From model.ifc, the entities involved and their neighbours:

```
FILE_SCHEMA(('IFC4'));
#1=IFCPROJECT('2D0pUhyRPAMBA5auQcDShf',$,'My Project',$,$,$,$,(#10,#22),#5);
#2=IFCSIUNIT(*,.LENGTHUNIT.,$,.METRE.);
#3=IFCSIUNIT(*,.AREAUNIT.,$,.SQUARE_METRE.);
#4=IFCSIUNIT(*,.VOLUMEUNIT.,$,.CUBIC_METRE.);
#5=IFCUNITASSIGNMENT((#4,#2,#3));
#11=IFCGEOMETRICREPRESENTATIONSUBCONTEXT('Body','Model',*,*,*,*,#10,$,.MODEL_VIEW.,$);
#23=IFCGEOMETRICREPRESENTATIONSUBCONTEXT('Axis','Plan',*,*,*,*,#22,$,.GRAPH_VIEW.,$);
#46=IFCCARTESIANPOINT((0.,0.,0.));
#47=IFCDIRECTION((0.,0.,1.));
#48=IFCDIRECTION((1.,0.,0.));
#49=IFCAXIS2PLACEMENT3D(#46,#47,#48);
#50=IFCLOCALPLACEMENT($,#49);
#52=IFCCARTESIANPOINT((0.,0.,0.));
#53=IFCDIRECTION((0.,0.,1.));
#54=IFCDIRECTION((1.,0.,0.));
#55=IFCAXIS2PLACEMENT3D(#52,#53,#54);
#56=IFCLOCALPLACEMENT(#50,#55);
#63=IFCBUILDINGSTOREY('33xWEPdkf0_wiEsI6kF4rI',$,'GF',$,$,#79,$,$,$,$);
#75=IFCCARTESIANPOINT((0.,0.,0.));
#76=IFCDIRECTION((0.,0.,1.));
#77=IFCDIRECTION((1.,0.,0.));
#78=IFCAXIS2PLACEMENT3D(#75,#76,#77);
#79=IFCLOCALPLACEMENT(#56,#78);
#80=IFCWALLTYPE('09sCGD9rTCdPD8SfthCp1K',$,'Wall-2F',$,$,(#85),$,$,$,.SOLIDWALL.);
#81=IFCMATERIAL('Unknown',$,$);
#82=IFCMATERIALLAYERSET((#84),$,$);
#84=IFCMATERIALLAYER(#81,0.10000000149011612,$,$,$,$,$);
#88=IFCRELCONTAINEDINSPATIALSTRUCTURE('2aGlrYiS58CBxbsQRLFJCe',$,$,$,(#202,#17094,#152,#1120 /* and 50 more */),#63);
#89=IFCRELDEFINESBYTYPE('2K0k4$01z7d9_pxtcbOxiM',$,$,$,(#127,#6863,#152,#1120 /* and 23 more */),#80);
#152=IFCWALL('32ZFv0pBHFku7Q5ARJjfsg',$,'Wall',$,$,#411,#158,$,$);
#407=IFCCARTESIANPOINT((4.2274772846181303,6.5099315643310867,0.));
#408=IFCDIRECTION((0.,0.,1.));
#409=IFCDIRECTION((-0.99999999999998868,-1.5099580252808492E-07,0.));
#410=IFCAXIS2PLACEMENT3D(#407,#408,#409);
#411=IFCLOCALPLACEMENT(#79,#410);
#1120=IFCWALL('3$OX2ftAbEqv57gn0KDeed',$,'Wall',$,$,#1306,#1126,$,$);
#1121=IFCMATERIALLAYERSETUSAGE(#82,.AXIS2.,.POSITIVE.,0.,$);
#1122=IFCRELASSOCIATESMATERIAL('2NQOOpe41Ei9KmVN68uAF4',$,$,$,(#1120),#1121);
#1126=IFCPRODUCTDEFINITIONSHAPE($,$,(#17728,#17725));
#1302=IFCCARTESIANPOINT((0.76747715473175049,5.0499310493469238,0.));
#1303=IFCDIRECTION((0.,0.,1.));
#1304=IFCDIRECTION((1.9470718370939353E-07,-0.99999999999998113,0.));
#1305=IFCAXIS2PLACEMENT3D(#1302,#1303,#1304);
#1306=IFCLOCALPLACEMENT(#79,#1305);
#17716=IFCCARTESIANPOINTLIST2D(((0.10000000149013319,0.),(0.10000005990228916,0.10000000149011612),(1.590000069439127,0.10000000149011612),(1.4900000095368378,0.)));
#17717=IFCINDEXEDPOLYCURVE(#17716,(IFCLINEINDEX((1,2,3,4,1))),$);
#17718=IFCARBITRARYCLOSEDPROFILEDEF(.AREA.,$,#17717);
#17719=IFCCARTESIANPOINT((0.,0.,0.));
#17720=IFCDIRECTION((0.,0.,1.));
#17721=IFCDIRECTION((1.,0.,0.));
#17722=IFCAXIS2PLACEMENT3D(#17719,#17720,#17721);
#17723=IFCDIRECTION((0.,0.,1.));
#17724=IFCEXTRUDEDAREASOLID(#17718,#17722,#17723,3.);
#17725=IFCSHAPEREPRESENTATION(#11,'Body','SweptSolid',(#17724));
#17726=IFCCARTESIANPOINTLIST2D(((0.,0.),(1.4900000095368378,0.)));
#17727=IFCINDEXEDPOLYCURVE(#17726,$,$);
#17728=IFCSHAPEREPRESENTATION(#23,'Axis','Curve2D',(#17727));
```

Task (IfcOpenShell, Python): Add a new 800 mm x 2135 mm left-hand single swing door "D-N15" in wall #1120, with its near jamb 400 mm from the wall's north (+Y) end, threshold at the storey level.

```python
import numpy as np
import ifcopenshell
import ifcopenshell.api.feature
import ifcopenshell.api.geometry
import ifcopenshell.api.root
import ifcopenshell.api.spatial
import ifcopenshell.geom
import ifcopenshell.util.element
import ifcopenshell.util.placement
import ifcopenshell.util.representation
import ifcopenshell.util.shape
import ifcopenshell.util.unit

model = ifcopenshell.open("model.ifc")
unit_scale = ifcopenshell.util.unit.calculate_unit_scale(model)
settings = ifcopenshell.geom.settings()


def volume(element):
    """Net volume in cubic metres, openings subtracted."""
    shape = ifcopenshell.geom.create_shape(settings, element)
    return ifcopenshell.util.shape.get_volume(shape.geometry)


wall = model.by_guid("3$OX2ftAbEqv57gn0KDeed")
storey = ifcopenshell.util.element.get_container(wall, ifc_class="IfcBuildingStorey")
context = ifcopenshell.util.representation.get_context(model, "Model", "Body", "MODEL_VIEW")
before = volume(wall)

width, height, from_end, sill = 0.8, 2.135, 0.4, 0.0  # metres

# The wall runs along its own X axis, and the end named is its -X end.
wall_shape = ifcopenshell.geom.create_shape(settings, wall)
x, y, z = ifcopenshell.util.shape.get_vertices(wall_shape.geometry).T
start = x.min() + from_end
face, thickness = float(y.min()), float(y.max() - y.min())
wall_matrix = ifcopenshell.util.placement.get_local_placement(wall.ObjectPlacement)
level = ifcopenshell.util.placement.get_local_placement(storey.ObjectPlacement)[2, 3]


def in_wall(x, y):
    """Placement at x, y metres in the wall's axes, at sill height."""
    matrix = wall_matrix.copy()
    matrix[:, 3] = wall_matrix @ np.array([x / unit_scale, y / unit_scale, 0.0, 1.0])
    matrix[2, 3] = level + sill / unit_scale
    return matrix


# Opening: a box that overshoots both wall faces by 50 mm.
opening = ifcopenshell.api.root.create_entity(model, ifc_class="IfcOpeningElement", predefined_type="OPENING")
box = ifcopenshell.api.geometry.add_wall_representation(
    model, context=context, length=width, height=height, thickness=thickness + 0.1
)
ifcopenshell.api.geometry.assign_representation(model, product=opening, representation=box)
ifcopenshell.api.geometry.edit_object_placement(model, product=opening, matrix=in_wall(start, face - 0.05), is_si=False)
ifcopenshell.api.feature.add_feature(model, feature=opening, element=wall)

door = ifcopenshell.api.root.create_entity(model, ifc_class="IfcDoor", name="D-N15", predefined_type="DOOR")
door.OverallWidth, door.OverallHeight = width / unit_scale, height / unit_scale
door.OperationType = "SINGLE_SWING_LEFT"
body = ifcopenshell.api.geometry.add_door_representation(
    model,
    context=context,
    overall_width=door.OverallWidth,
    overall_height=door.OverallHeight,
    operation_type="SINGLE_SWING_LEFT",
    lining_properties={"LiningDepth": thickness / unit_scale, "ThresholdDepth": thickness / unit_scale},
)
ifcopenshell.api.geometry.assign_representation(model, product=door, representation=body)
ifcopenshell.api.spatial.assign_container(model, products=[door], relating_structure=storey)
ifcopenshell.api.feature.add_filling(model, opening=opening, element=door)

# The lining spans the wall, so the door starts at the wall face.
ifcopenshell.api.geometry.edit_object_placement(model, product=door, matrix=in_wall(start, face), is_si=False)

after = volume(wall)

print(f"wall volume {before:.3f} -> {after:.3f} m3")

model.write("model-out.ifc")
```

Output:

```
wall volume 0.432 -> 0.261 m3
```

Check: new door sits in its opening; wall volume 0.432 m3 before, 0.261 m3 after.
